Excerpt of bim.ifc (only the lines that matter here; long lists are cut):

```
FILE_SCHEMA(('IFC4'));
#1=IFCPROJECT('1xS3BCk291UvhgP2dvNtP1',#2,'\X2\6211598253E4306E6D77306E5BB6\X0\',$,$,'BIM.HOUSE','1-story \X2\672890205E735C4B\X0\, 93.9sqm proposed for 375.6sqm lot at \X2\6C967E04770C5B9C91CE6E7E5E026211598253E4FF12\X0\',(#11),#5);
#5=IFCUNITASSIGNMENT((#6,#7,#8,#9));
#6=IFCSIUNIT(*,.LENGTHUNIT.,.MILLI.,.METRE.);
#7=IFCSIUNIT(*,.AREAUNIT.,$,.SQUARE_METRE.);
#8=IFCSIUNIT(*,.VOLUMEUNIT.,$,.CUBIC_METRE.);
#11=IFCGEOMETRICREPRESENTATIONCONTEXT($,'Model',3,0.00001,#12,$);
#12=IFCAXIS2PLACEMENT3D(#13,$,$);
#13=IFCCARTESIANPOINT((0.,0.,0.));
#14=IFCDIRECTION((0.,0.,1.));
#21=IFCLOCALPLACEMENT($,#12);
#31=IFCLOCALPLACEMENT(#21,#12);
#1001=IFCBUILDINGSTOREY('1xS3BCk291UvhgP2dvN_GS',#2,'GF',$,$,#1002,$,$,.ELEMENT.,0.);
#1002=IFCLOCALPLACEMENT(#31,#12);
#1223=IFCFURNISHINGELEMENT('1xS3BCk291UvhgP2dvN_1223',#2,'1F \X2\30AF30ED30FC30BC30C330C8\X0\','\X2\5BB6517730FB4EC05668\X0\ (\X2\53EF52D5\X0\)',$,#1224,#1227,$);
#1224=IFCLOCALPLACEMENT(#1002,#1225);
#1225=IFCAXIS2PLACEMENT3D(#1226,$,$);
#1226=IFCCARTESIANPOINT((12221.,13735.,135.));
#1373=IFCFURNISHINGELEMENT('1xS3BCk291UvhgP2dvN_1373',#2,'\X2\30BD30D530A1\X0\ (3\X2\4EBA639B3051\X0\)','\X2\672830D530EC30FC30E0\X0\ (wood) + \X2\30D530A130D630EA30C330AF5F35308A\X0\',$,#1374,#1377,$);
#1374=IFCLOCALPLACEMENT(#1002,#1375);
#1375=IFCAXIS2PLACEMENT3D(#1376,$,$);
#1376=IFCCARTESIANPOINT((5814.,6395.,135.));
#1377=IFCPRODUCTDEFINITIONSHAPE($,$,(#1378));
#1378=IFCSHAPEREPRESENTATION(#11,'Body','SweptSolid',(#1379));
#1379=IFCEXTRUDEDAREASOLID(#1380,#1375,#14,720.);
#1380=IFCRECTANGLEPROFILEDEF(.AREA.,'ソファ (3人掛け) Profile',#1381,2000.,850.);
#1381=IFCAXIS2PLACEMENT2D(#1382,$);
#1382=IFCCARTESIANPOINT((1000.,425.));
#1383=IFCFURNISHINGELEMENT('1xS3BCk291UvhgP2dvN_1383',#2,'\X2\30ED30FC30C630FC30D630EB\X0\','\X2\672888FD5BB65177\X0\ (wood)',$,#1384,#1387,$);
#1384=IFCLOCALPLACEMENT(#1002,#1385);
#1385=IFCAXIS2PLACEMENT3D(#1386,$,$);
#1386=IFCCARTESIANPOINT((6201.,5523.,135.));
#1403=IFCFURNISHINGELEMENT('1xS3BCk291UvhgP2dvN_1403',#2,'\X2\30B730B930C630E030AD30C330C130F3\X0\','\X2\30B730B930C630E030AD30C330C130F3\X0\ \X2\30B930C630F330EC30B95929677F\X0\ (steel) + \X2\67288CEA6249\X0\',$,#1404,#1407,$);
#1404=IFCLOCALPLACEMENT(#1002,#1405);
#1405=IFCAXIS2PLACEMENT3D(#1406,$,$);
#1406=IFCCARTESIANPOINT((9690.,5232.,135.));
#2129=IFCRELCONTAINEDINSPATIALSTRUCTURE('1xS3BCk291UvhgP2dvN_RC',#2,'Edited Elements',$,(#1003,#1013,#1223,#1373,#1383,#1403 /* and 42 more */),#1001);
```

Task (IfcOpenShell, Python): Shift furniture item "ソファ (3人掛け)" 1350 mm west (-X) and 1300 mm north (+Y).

```python
import ifcopenshell
import ifcopenshell.api.geometry
import ifcopenshell.util.placement
import ifcopenshell.util.unit

model = ifcopenshell.open("bim.ifc")
unit_scale = ifcopenshell.util.unit.calculate_unit_scale(model)

item = model.by_guid("1xS3BCk291UvhgP2dvN_1373")
matrix = ifcopenshell.util.placement.get_local_placement(item.ObjectPlacement)
matrix[0, 3] -= 1.35 / unit_scale
matrix[1, 3] += 1.3 / unit_scale
ifcopenshell.api.geometry.edit_object_placement(model, product=item, matrix=matrix, is_si=False)

print(ifcopenshell.util.placement.get_local_placement(item.ObjectPlacement).round(3) + 0.0)

model.write("bim_updated.ifc")
```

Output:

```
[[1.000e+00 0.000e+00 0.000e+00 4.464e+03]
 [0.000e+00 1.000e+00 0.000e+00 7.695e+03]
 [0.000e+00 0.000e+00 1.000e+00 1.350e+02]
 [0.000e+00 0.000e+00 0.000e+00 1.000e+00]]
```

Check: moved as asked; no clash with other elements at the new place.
